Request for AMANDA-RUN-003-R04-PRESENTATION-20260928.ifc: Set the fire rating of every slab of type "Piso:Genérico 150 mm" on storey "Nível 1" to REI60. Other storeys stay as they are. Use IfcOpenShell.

First a look at what the model holds.

```python
import ifcopenshell
import ifcopenshell.util.element

model = ifcopenshell.open("AMANDA-RUN-003-R04-PRESENTATION-20260928.ifc")
print(model.schema)
storey = next(s for s in model.by_type("IfcBuildingStorey") if s.Name == "Nível 1")
slabs = [e for e in ifcopenshell.util.element.get_decomposition(storey) if e.is_a("IfcSlab")]
seen = {}
for e in slabs:
    element_type = ifcopenshell.util.element.get_type(e)
    key = (element_type.Name if element_type != e and element_type else None, ifcopenshell.util.element.get_pset(e, "Pset_SlabCommon", "FireRating"))
    seen[key] = seen.get(key, 0) + 1
for (name, value), count in sorted(seen.items(), key=str):
    print(count, "x", name, "|", value)
```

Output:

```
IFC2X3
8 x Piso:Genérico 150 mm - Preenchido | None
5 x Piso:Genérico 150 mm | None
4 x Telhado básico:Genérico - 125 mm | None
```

```python
import ifcopenshell
import ifcopenshell.api.pset
import ifcopenshell.util.element

model = ifcopenshell.open("AMANDA-RUN-003-R04-PRESENTATION-20260928.ifc")

storey = next(s for s in model.by_type("IfcBuildingStorey") if s.Name == "Nível 1")
slabs = [e for e in ifcopenshell.util.element.get_decomposition(storey) if e.is_a("IfcSlab")]

count = 0
for e in slabs:
    element_type = ifcopenshell.util.element.get_type(e)
    if element_type in (None, e) or element_type.Name != "Piso:Genérico 150 mm":
        continue
    # add_pset returns the element's existing set when there is one.
    pset = ifcopenshell.api.pset.add_pset(model, product=e, name="Pset_SlabCommon")
    ifcopenshell.api.pset.edit_pset(model, pset=pset, properties={"FireRating": "REI60"})
    count += 1

print(count, "slabs updated")

model.write("AMANDA-RUN-003-R04-PRESENTATION-20260928_rev.ifc")
```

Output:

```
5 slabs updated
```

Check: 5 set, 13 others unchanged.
